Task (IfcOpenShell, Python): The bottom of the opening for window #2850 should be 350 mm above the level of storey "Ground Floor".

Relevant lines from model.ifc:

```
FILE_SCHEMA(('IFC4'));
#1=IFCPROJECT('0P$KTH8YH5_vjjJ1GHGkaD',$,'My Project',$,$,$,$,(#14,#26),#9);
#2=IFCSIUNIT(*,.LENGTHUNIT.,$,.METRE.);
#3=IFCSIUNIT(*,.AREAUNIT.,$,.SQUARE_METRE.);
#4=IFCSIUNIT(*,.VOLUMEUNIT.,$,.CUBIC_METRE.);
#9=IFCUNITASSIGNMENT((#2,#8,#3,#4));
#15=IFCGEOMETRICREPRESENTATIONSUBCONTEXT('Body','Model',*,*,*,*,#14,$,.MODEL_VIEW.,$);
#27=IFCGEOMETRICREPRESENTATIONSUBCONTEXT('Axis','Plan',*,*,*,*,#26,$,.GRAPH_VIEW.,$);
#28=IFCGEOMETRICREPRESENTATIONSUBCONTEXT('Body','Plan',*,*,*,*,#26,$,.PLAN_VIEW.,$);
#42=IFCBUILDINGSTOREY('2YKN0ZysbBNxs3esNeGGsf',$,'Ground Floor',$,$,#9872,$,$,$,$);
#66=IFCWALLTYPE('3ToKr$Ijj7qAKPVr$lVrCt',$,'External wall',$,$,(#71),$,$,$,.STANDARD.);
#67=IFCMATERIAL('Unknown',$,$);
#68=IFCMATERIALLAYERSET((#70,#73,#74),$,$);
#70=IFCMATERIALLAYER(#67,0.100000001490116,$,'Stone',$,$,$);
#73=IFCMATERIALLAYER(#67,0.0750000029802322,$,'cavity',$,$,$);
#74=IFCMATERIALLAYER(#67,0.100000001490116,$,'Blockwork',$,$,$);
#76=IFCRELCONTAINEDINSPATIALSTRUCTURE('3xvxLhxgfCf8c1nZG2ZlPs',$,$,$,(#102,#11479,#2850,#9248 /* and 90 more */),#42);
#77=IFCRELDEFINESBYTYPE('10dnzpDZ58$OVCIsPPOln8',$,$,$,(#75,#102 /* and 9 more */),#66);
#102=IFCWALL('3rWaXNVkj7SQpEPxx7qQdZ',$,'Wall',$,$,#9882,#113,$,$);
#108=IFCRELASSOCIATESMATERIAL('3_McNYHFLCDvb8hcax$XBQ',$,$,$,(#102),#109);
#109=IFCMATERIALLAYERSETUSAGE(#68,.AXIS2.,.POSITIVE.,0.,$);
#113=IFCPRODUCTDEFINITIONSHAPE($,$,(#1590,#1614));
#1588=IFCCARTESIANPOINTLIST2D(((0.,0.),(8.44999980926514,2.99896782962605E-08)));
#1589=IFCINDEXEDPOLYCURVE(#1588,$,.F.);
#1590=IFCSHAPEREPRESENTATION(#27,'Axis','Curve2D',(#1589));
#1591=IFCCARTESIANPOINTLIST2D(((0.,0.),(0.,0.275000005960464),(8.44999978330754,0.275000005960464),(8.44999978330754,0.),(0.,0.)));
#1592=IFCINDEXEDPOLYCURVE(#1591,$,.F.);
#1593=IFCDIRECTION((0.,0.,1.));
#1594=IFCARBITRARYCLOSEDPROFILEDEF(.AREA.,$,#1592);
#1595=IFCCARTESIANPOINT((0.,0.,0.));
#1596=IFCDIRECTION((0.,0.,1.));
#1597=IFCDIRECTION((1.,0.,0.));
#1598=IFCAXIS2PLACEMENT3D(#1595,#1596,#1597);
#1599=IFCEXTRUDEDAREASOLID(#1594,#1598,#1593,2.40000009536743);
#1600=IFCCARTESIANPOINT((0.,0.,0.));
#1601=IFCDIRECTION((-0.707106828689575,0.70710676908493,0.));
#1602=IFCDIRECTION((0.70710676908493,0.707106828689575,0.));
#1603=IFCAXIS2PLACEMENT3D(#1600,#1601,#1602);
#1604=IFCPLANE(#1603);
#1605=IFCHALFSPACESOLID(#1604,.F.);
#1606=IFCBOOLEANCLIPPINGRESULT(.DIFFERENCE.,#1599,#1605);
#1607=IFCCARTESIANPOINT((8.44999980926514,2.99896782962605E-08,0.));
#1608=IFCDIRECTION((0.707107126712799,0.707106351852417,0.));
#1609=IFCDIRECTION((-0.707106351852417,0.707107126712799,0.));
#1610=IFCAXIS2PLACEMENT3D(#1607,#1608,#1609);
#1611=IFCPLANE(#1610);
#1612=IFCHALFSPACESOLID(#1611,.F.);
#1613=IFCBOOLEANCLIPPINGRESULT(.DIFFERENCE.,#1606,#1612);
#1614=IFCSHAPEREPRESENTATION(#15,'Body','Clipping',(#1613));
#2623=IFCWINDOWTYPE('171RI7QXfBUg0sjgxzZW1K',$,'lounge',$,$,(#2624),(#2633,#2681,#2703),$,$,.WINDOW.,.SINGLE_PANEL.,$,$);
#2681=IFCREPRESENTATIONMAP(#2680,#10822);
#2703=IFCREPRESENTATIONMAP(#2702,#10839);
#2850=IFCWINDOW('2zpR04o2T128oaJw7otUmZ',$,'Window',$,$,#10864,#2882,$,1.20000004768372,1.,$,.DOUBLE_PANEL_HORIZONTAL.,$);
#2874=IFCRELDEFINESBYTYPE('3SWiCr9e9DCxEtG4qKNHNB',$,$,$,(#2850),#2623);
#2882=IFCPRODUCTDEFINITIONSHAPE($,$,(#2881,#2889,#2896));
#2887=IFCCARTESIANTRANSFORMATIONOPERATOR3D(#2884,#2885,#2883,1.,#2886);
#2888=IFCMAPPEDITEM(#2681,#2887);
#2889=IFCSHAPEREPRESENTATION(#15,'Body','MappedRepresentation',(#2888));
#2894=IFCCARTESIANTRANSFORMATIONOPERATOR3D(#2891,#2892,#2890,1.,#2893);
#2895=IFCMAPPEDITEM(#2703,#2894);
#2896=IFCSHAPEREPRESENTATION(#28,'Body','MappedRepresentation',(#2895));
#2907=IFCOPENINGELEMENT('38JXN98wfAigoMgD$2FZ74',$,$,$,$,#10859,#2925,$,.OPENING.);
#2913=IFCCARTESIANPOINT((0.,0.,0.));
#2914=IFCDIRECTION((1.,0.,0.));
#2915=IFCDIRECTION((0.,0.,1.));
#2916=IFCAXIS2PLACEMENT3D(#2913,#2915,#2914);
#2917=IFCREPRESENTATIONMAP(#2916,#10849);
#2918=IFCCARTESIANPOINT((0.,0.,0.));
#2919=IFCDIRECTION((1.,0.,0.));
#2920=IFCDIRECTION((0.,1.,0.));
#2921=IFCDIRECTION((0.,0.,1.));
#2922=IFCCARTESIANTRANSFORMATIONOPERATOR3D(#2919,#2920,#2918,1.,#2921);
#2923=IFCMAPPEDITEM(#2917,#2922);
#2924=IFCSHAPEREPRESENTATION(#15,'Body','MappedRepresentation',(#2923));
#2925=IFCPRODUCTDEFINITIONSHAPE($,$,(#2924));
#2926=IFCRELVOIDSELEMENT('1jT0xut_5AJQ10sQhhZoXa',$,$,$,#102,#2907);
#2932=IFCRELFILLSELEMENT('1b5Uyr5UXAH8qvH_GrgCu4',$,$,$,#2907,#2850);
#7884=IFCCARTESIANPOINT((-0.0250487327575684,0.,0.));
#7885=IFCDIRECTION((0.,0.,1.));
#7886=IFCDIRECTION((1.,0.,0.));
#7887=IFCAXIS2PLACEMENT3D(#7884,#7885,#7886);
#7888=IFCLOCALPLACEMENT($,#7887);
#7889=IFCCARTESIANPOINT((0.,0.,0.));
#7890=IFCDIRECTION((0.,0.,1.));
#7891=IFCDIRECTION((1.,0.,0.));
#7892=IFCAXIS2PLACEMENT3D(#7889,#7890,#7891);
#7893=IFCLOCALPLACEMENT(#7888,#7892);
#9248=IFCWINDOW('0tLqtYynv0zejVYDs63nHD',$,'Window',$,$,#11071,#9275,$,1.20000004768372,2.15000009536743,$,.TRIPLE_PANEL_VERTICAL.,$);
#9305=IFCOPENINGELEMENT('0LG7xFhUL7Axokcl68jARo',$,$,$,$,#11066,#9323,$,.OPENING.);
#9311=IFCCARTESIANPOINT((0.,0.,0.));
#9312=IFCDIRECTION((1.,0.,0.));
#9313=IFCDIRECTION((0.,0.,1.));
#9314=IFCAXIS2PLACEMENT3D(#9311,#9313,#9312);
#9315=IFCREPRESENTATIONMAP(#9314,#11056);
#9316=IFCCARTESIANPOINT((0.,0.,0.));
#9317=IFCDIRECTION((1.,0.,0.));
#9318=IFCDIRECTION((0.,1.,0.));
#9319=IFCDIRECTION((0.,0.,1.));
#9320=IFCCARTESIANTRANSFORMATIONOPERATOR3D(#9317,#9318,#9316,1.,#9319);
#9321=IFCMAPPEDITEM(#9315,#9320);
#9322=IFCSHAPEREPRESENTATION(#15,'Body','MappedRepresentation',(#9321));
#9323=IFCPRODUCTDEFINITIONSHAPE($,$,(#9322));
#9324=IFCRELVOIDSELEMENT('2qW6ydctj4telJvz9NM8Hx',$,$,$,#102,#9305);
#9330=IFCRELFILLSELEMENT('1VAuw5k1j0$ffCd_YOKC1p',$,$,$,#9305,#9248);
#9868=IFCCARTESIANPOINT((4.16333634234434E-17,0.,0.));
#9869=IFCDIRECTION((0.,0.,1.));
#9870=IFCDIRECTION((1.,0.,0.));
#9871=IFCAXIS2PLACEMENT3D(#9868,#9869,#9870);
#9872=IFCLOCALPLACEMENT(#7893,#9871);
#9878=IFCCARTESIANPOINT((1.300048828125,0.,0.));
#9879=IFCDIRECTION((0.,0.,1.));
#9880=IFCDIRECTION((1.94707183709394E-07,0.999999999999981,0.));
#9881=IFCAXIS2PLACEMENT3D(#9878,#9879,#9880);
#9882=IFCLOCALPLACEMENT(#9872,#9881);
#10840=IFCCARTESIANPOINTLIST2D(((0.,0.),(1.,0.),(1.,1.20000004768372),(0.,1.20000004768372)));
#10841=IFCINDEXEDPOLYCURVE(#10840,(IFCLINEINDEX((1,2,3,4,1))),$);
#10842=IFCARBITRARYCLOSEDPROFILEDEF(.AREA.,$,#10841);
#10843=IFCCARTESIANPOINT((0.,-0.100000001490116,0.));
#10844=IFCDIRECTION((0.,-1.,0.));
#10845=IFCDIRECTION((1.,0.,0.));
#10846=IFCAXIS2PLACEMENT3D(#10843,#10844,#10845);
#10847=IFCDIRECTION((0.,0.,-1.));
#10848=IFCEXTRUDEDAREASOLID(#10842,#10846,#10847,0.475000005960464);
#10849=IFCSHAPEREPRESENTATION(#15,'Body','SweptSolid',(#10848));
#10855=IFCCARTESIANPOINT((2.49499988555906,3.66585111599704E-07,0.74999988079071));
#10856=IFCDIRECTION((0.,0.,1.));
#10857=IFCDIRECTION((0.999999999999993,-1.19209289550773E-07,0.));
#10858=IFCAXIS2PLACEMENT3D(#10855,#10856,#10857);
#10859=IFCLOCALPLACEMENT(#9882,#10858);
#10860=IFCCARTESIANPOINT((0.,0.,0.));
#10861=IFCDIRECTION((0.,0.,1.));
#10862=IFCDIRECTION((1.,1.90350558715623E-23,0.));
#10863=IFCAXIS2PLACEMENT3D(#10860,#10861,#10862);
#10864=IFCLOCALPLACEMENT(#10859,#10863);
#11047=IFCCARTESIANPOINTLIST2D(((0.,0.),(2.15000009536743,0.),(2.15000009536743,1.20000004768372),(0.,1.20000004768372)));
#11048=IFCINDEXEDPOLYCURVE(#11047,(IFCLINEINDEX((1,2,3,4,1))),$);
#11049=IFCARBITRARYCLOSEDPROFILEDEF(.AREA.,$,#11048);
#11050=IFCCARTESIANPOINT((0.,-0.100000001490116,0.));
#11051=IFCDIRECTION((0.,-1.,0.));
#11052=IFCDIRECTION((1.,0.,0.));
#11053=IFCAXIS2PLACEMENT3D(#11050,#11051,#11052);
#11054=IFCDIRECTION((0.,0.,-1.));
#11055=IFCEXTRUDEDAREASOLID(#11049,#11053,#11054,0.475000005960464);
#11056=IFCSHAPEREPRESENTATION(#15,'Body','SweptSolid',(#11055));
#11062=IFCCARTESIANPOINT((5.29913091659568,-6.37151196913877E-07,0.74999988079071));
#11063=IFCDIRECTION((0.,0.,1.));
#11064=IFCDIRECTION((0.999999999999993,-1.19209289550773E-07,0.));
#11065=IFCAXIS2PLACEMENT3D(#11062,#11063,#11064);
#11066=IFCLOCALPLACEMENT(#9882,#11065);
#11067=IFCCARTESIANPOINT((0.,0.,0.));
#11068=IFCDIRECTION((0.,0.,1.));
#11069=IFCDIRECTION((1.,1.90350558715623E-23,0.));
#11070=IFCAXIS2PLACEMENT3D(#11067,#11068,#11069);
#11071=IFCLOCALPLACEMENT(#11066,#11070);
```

```python
import numpy as np
import ifcopenshell
import ifcopenshell.api.geometry
import ifcopenshell.geom
import ifcopenshell.util.element
import ifcopenshell.util.placement
import ifcopenshell.util.shape
import ifcopenshell.util.unit

model = ifcopenshell.open("model.ifc")
unit_scale = ifcopenshell.util.unit.calculate_unit_scale(model)

window = model.by_guid("2zpR04o2T128oaJw7otUmZ")
opening = window.FillsVoids[0].RelatingOpeningElement
storey = ifcopenshell.util.element.get_container(window, ifc_class="IfcBuildingStorey")
level = ifcopenshell.util.placement.get_local_placement(storey.ObjectPlacement)[2, 3]

# The opening's origin need not be at the sill, so measure its lowest point.
shape = ifcopenshell.geom.create_shape(ifcopenshell.geom.settings(), opening)
bottom = ifcopenshell.util.shape.get_shape_bottom_elevation(shape, shape.geometry) / unit_scale
dz = level + 0.35 / unit_scale - bottom

shift = np.array([0.0, 0.0, dz])
# The window is placed relative to its opening, so it follows when the opening moves.
matrix = ifcopenshell.util.placement.get_local_placement(opening.ObjectPlacement)
matrix[:3, 3] += shift
ifcopenshell.api.geometry.edit_object_placement(
    model, product=opening, matrix=matrix, is_si=False, should_transform_children=True
)

print(f"moved by {dz * unit_scale:+.3f} m")

model.write("model_updated.ifc")
```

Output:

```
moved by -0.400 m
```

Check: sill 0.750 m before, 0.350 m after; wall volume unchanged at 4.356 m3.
